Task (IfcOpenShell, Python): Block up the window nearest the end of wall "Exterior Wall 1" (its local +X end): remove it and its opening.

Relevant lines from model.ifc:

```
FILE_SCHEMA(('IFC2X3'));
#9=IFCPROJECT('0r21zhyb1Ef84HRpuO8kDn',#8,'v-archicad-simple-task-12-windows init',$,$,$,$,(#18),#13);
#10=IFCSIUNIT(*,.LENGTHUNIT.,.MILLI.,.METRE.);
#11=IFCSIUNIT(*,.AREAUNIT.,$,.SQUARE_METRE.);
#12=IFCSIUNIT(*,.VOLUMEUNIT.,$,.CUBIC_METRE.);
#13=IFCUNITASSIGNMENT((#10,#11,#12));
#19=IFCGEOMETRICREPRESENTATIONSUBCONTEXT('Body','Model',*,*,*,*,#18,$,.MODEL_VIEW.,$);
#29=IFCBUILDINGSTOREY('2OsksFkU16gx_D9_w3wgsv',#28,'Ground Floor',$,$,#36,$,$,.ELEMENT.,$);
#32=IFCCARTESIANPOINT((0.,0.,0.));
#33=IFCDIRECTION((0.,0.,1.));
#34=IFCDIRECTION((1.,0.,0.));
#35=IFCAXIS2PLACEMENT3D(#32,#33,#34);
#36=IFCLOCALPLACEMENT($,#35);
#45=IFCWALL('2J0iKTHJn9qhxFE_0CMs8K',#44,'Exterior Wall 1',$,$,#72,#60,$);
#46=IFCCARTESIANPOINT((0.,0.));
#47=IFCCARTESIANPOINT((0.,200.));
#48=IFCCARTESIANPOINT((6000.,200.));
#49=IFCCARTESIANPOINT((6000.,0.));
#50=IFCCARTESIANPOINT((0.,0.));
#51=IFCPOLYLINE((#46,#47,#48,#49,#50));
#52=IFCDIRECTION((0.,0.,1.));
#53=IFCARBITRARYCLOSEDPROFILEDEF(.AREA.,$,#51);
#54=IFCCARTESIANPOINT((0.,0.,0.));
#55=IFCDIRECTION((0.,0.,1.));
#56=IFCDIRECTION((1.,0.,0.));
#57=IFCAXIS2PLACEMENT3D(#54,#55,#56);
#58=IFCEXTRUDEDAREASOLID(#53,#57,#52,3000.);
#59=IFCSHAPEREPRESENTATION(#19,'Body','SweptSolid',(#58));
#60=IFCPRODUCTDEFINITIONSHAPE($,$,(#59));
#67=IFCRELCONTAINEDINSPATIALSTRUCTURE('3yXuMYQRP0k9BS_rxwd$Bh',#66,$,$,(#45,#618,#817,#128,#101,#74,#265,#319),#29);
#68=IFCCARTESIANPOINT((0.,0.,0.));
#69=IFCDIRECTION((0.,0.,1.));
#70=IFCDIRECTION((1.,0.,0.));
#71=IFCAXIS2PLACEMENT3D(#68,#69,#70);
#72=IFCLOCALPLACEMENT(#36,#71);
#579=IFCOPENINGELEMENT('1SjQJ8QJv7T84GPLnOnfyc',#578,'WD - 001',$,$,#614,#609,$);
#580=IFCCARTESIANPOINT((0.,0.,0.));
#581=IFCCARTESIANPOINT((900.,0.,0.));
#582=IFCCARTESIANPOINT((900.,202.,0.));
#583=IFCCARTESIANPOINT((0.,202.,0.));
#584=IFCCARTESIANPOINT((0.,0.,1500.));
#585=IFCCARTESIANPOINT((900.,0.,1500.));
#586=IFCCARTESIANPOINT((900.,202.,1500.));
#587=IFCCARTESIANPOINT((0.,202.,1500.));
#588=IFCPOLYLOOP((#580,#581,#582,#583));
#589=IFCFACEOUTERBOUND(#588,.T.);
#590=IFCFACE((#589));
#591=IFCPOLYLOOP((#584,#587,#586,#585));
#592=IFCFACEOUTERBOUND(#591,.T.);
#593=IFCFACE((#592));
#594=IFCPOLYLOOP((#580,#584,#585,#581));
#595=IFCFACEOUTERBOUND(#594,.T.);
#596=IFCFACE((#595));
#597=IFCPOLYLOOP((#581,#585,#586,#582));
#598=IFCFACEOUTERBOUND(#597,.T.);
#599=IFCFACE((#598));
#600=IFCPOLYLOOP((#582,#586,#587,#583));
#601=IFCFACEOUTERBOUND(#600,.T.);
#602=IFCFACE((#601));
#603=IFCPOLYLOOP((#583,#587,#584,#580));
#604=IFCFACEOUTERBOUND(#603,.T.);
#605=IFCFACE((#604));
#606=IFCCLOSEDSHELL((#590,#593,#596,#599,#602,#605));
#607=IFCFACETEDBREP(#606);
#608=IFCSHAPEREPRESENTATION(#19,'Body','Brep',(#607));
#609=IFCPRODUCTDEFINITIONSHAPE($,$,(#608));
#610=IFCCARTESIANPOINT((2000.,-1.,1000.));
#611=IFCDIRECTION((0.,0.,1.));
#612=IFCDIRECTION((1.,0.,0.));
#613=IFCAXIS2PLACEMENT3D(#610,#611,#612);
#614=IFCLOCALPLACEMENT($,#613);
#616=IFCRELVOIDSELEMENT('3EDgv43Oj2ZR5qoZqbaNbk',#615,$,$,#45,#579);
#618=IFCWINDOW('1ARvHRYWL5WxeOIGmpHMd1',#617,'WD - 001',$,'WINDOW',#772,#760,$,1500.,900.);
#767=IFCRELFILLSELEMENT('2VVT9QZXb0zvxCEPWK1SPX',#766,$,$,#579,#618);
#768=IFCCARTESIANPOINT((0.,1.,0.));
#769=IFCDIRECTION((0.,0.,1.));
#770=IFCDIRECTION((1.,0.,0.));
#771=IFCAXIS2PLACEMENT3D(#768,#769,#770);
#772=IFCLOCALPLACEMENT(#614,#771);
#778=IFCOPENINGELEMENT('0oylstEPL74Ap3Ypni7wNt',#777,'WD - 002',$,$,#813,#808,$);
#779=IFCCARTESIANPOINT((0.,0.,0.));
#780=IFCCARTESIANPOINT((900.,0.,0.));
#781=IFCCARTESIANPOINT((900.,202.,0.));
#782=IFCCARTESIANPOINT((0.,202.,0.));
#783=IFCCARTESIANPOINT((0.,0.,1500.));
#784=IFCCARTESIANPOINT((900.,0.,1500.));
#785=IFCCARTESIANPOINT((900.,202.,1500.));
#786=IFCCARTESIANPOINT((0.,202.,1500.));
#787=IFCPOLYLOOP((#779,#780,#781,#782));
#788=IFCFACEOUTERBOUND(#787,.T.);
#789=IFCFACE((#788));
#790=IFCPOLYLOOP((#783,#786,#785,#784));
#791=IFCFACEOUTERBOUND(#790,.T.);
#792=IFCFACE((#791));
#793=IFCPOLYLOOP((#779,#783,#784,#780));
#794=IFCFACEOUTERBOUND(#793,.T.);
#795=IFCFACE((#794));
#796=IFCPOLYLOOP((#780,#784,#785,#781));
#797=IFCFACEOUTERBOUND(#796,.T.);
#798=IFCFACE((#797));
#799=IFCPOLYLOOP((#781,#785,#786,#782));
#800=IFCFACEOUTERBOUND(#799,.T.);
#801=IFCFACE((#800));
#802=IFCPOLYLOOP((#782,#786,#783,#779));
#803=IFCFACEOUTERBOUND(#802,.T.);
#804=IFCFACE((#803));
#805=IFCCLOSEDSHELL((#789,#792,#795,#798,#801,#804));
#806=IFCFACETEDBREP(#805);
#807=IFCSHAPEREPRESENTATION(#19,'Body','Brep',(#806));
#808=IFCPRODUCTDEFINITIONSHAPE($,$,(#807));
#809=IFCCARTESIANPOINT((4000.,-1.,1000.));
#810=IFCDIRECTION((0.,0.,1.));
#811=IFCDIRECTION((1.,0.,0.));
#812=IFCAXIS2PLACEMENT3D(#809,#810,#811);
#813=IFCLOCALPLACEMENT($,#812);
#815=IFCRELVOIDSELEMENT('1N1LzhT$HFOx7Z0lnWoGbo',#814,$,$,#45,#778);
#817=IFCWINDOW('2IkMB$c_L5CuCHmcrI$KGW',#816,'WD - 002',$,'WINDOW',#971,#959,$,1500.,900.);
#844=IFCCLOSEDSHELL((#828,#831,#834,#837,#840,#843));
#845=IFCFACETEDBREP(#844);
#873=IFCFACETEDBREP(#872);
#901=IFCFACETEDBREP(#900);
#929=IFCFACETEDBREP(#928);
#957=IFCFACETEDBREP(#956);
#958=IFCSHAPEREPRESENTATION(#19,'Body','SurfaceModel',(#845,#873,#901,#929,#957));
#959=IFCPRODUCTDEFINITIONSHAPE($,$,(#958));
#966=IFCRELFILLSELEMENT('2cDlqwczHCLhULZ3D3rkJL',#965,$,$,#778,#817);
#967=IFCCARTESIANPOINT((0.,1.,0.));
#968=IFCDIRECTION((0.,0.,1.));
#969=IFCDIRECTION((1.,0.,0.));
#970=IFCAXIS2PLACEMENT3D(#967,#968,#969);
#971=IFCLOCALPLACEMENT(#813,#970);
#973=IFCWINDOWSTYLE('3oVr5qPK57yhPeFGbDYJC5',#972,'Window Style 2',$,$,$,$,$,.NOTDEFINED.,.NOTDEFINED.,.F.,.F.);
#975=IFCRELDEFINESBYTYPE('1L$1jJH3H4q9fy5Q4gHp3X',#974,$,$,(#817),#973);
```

```python
import ifcopenshell
import ifcopenshell.api.feature
import ifcopenshell.api.root
import ifcopenshell.geom
import ifcopenshell.util.shape

model = ifcopenshell.open("model.ifc")
settings = ifcopenshell.geom.settings()


def volume(element):
    """Net volume in cubic metres, openings subtracted."""
    shape = ifcopenshell.geom.create_shape(settings, element)
    return ifcopenshell.util.shape.get_volume(shape.geometry)


window = model.by_id(817)
opening = window.FillsVoids[0].RelatingOpeningElement
wall = opening.VoidsElements[0].RelatingBuildingElement
before = volume(wall)

ifcopenshell.api.root.remove_product(model, product=window)
ifcopenshell.api.feature.remove_feature(model, feature=opening)

after = volume(wall)

print(f"wall volume {before:.3f} -> {after:.3f} m3")

model.write("model_v2.ifc")
```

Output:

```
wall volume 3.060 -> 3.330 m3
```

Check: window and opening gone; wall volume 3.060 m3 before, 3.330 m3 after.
